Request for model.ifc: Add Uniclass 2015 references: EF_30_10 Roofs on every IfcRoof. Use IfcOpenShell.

First a look at what the model holds.

```python
import ifcopenshell

model = ifcopenshell.open("model.ifc")
print(model.schema)
print("classifications:", [c.Name for c in model.by_type("IfcClassification")])
for ifc_class in ("IfcDoor", "IfcRoof", "IfcStair", "IfcWall", "IfcWindow"):
    print(ifc_class, len(model.by_type(ifc_class)))
```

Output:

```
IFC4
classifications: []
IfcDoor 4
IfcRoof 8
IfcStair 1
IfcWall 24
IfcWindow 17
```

```python
import ifcopenshell
import ifcopenshell.api.classification

model = ifcopenshell.open("model.ifc")

system = ifcopenshell.api.classification.add_classification(model, classification="Uniclass 2015")

codes = {
    "IfcRoof": ("EF_30_10", "Roofs"),
}
for ifc_class, (code, name) in codes.items():
    products = model.by_type(ifc_class)
    ifcopenshell.api.classification.add_reference(
        model, products=products, classification=system, identification=code, name=name
    )
    print(code, len(products))

model.write("model_updated.ifc")
```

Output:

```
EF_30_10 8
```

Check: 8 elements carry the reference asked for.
